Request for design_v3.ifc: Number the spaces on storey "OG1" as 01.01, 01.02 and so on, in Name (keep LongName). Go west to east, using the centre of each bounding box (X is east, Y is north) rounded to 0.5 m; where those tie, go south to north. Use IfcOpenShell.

First a look at what the model holds.

```python
import ifcopenshell
import ifcopenshell.util.element
import ifcopenshell.util.placement

model = ifcopenshell.open("design_v3.ifc")
print(model.schema)
storey = next(s for s in model.by_type("IfcBuildingStorey") if s.Name == "OG1")
spaces = [e for e in ifcopenshell.util.element.get_decomposition(storey) if e.is_a("IfcSpace")]
for e in sorted(spaces, key=lambda e: e.id()):
    origin = ifcopenshell.util.placement.get_local_placement(e.ObjectPlacement)[:3, 3]
    print(e.id(), e.Name, e.LongName, origin.round(2) + 0.0, sep=" | ")
```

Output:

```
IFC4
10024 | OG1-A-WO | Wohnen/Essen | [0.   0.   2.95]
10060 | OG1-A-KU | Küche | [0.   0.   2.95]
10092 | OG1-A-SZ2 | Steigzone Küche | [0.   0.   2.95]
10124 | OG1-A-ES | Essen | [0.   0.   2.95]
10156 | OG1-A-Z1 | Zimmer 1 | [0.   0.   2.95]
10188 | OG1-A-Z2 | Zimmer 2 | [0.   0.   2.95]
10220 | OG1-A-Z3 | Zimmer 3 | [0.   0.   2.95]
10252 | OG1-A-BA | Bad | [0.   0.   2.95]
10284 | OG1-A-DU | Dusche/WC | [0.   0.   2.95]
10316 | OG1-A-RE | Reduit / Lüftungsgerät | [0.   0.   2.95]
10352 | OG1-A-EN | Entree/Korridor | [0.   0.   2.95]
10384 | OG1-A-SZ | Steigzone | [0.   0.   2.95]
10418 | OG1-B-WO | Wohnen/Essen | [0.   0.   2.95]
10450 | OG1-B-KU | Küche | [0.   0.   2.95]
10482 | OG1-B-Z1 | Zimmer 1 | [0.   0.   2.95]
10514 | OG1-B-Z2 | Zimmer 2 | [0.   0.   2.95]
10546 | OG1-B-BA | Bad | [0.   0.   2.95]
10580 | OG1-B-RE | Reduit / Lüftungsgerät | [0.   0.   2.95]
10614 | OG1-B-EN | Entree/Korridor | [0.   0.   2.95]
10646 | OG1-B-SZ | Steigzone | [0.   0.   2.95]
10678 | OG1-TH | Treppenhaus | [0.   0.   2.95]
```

```python
import ifcopenshell
import ifcopenshell.geom
import ifcopenshell.util.element
import ifcopenshell.util.shape

model = ifcopenshell.open("design_v3.ifc")
settings = ifcopenshell.geom.settings()
settings.set("use-world-coords", True)


def centre(element):
    shape = ifcopenshell.geom.create_shape(settings, element)
    return ifcopenshell.util.shape.get_bbox_centroid(shape.geometry)


storey = next(s for s in model.by_type("IfcBuildingStorey") if s.Name == "OG1")
spaces = [e for e in ifcopenshell.util.element.get_decomposition(storey) if e.is_a("IfcSpace")]

# Insertion points can sit at a corner or the storey origin, so sort by the geometry (in metres).
centres = {e: centre(e) for e in spaces}
spaces.sort(key=lambda e: (round(centres[e][0] / 0.5), centres[e][1]))

for i, e in enumerate(spaces, start=1):
    number = f"01.{i:02d}"
    e.Name = number
    print(e.id(), number)

model.write("design_v3-out.ifc")
```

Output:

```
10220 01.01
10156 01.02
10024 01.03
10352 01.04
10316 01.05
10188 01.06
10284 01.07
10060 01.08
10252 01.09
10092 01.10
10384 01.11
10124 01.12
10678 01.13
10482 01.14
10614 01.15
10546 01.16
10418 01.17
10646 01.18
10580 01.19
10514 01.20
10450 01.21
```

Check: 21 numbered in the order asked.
